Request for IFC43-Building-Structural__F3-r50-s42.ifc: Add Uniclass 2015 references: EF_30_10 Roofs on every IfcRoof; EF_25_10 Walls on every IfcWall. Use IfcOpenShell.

First a look at what the model holds.

```python
import ifcopenshell

model = ifcopenshell.open("IFC43-Building-Structural__F3-r50-s42.ifc")
print(model.schema)
print("classifications:", [c.Name for c in model.by_type("IfcClassification")])
for ifc_class in ("IfcDoor", "IfcRoof", "IfcStair", "IfcWall", "IfcWindow"):
    print(ifc_class, len(model.by_type(ifc_class)))
```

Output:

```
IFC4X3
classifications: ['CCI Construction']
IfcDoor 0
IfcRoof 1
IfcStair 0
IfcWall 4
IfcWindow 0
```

```python
import ifcopenshell
import ifcopenshell.api.classification

model = ifcopenshell.open("IFC43-Building-Structural__F3-r50-s42.ifc")

system = ifcopenshell.api.classification.add_classification(model, classification="Uniclass 2015")

codes = {
    "IfcRoof": ("EF_30_10", "Roofs"),
    "IfcWall": ("EF_25_10", "Walls"),
}
for ifc_class, (code, name) in codes.items():
    products = model.by_type(ifc_class)
    ifcopenshell.api.classification.add_reference(
        model, products=products, classification=system, identification=code, name=name
    )
    print(code, len(products))

model.write("IFC43-Building-Structural__F3-r50-s42_updated.ifc")
```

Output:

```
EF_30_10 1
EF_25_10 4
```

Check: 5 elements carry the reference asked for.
